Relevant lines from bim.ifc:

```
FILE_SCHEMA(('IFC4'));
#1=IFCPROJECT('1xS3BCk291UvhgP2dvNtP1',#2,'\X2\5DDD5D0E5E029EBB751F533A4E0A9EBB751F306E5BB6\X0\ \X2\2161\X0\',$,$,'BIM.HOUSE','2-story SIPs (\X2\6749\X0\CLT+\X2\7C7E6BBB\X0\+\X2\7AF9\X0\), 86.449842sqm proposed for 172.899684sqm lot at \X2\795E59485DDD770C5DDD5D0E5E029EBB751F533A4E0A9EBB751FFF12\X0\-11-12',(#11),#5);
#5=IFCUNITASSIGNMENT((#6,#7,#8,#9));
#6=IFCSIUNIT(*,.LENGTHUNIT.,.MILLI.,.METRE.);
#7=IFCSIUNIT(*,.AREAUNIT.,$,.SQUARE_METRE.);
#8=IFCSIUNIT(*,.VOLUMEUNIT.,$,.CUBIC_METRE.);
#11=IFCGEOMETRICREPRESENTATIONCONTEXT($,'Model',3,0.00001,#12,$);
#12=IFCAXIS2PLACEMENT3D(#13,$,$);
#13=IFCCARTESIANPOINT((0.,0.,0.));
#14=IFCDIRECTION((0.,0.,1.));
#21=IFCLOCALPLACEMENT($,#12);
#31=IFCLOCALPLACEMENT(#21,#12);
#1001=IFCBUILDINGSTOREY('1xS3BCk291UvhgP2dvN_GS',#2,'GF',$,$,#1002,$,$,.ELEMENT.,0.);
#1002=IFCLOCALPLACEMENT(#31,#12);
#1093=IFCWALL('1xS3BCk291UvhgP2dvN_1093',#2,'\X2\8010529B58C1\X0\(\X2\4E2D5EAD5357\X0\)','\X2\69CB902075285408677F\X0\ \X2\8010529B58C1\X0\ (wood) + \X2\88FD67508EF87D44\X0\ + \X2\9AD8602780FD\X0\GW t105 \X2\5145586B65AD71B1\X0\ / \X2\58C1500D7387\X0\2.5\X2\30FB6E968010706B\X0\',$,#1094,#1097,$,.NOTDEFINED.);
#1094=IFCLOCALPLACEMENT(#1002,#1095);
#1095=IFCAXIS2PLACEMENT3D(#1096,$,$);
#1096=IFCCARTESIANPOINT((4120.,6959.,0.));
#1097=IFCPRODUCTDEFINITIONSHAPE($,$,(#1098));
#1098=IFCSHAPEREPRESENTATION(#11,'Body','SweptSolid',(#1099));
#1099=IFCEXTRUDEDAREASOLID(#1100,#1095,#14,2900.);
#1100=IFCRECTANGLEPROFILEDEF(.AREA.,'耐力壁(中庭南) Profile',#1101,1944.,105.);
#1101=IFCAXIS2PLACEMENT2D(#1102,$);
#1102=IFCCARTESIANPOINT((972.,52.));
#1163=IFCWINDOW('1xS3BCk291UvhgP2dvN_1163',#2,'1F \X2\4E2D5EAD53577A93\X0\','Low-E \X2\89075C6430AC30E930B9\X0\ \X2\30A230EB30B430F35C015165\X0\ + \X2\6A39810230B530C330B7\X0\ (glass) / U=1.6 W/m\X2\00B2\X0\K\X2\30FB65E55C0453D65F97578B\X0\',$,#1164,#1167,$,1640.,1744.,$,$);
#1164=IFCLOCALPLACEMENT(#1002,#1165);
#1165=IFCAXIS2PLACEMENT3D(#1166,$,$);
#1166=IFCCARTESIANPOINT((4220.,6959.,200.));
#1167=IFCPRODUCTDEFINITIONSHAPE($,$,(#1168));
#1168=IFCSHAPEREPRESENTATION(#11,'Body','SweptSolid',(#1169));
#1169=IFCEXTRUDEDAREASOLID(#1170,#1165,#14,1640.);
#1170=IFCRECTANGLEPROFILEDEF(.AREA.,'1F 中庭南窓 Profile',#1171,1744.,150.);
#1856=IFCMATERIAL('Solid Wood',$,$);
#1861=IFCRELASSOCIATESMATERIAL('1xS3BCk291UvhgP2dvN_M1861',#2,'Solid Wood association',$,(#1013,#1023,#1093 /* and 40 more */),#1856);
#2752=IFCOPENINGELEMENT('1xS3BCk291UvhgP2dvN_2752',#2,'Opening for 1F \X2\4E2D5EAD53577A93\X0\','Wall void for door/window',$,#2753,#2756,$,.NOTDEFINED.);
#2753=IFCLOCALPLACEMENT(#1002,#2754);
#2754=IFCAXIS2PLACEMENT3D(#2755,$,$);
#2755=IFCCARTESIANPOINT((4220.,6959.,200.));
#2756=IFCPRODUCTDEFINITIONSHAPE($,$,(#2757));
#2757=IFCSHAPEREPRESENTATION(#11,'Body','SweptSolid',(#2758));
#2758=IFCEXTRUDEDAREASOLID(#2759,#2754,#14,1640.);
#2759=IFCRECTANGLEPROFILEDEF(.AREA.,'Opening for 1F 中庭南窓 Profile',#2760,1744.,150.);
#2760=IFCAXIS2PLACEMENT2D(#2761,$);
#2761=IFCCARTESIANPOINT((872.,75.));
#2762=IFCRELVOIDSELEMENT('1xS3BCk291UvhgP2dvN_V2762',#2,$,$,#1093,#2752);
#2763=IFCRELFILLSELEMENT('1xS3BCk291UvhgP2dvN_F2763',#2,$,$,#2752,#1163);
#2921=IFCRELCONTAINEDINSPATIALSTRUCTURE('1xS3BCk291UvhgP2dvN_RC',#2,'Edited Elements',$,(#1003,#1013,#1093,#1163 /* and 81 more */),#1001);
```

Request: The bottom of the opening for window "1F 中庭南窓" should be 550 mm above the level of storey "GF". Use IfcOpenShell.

```python
import numpy as np
import ifcopenshell
import ifcopenshell.api.geometry
import ifcopenshell.geom
import ifcopenshell.util.element
import ifcopenshell.util.placement
import ifcopenshell.util.shape
import ifcopenshell.util.unit

model = ifcopenshell.open("bim.ifc")
unit_scale = ifcopenshell.util.unit.calculate_unit_scale(model)

window = model.by_guid("1xS3BCk291UvhgP2dvN_1163")
opening = window.FillsVoids[0].RelatingOpeningElement
storey = ifcopenshell.util.element.get_container(window, ifc_class="IfcBuildingStorey")
level = ifcopenshell.util.placement.get_local_placement(storey.ObjectPlacement)[2, 3]

# The opening's origin need not be at the sill, so measure its lowest point.
shape = ifcopenshell.geom.create_shape(ifcopenshell.geom.settings(), opening)
bottom = ifcopenshell.util.shape.get_shape_bottom_elevation(shape, shape.geometry) / unit_scale
dz = level + 550.0 - bottom

shift = np.array([0.0, 0.0, dz])
# The window is not placed relative to its opening, so move both.
for product in (opening, window):
    matrix = ifcopenshell.util.placement.get_local_placement(product.ObjectPlacement)
    matrix[:3, 3] += shift
    ifcopenshell.api.geometry.edit_object_placement(model, product=product, matrix=matrix, is_si=False)

print(f"moved by {dz * unit_scale:+.3f} m")

model.write("bim_v2.ifc")
```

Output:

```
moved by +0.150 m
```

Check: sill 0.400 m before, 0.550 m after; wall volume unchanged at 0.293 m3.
